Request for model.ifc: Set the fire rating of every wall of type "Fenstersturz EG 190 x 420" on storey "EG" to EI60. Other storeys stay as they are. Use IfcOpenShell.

First a look at what the model holds.

```python
import ifcopenshell
import ifcopenshell.util.element

model = ifcopenshell.open("model.ifc")
print(model.schema)
storey = next(s for s in model.by_type("IfcBuildingStorey") if s.Name == "EG")
walls = [e for e in ifcopenshell.util.element.get_decomposition(storey) if e.is_a("IfcWall")]
seen = {}
for e in walls:
    element_type = ifcopenshell.util.element.get_type(e)
    key = (element_type.Name if element_type != e and element_type else None, ifcopenshell.util.element.get_pset(e, "Pset_WallCommon", "FireRating"))
    seen[key] = seen.get(key, 0) + 1
for (name, value), count in sorted(seen.items(), key=str):
    print(count, "x", name, "|", value)
```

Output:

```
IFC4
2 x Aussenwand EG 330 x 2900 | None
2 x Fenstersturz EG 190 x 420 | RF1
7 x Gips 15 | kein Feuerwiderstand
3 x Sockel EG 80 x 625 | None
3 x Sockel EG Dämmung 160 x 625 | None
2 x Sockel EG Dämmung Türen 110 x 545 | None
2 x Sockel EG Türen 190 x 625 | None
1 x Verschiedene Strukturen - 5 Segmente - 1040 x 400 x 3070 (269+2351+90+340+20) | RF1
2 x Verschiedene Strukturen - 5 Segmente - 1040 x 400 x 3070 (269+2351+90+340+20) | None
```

```python
import ifcopenshell
import ifcopenshell.api.pset
import ifcopenshell.util.element

model = ifcopenshell.open("model.ifc")

storey = next(s for s in model.by_type("IfcBuildingStorey") if s.Name == "EG")
walls = [e for e in ifcopenshell.util.element.get_decomposition(storey) if e.is_a("IfcWall")]

count = 0
for e in walls:
    element_type = ifcopenshell.util.element.get_type(e)
    if element_type in (None, e) or element_type.Name != "Fenstersturz EG 190 x 420":
        continue
    # add_pset returns the element's existing set when there is one.
    pset = ifcopenshell.api.pset.add_pset(model, product=e, name="Pset_WallCommon")
    ifcopenshell.api.pset.edit_pset(model, pset=pset, properties={"FireRating": "EI60"})
    count += 1

print(count, "walls updated")

model.write("model_v2.ifc")
```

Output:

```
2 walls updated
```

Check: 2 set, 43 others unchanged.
